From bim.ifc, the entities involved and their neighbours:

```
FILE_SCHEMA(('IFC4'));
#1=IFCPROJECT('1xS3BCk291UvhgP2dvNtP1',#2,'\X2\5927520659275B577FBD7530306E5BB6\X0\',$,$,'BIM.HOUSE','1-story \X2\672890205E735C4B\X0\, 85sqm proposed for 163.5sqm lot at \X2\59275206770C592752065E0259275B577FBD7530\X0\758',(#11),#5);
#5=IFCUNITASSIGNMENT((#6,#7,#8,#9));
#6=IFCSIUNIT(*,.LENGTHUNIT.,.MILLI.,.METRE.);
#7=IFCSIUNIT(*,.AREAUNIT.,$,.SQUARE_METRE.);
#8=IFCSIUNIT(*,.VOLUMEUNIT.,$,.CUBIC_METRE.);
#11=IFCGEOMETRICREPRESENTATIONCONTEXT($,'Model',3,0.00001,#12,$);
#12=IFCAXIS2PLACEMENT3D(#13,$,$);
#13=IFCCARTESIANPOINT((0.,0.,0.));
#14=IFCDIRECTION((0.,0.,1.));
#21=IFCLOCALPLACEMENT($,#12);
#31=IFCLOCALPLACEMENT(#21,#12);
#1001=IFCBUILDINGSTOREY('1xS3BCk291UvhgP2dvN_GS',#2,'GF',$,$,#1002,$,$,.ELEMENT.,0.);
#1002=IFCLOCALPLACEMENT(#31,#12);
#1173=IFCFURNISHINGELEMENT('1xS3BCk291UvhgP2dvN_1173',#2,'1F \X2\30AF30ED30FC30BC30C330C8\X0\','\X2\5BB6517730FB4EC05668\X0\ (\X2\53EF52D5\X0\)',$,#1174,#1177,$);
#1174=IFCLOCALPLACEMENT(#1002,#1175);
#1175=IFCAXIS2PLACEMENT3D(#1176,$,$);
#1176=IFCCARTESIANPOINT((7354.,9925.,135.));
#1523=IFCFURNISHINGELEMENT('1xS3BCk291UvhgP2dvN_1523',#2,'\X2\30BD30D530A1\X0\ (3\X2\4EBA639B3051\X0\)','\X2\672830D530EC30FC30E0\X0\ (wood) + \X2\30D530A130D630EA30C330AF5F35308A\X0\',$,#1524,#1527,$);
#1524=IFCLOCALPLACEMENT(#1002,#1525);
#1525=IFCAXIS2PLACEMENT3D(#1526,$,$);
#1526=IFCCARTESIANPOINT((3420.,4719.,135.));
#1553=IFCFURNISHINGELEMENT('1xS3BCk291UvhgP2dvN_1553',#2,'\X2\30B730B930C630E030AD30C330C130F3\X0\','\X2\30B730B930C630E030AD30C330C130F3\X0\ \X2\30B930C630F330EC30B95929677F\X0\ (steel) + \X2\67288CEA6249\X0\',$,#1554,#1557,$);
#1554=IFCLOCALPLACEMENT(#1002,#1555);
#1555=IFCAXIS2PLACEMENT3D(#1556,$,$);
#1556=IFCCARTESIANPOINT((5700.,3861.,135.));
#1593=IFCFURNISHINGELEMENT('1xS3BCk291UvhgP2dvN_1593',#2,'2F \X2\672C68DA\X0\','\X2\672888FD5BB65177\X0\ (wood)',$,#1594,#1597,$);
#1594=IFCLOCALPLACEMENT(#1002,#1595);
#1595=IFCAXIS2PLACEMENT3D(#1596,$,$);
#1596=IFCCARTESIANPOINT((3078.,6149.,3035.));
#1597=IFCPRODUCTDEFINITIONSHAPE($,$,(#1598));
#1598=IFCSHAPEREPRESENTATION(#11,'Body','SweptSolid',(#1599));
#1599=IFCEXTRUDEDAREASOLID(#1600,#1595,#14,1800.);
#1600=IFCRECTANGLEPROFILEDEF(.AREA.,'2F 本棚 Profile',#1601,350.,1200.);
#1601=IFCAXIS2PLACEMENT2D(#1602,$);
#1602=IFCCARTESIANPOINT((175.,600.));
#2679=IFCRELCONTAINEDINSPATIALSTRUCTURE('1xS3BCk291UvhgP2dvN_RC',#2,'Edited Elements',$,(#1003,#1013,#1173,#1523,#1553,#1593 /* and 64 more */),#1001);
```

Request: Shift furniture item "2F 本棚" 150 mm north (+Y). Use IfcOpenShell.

```python
import ifcopenshell
import ifcopenshell.api.geometry
import ifcopenshell.util.placement
import ifcopenshell.util.unit

model = ifcopenshell.open("bim.ifc")
unit_scale = ifcopenshell.util.unit.calculate_unit_scale(model)

item = model.by_guid("1xS3BCk291UvhgP2dvN_1593")
matrix = ifcopenshell.util.placement.get_local_placement(item.ObjectPlacement)
matrix[1, 3] += 0.15 / unit_scale
ifcopenshell.api.geometry.edit_object_placement(model, product=item, matrix=matrix, is_si=False)

print(ifcopenshell.util.placement.get_local_placement(item.ObjectPlacement).round(3) + 0.0)

model.write("bim_updated.ifc")
```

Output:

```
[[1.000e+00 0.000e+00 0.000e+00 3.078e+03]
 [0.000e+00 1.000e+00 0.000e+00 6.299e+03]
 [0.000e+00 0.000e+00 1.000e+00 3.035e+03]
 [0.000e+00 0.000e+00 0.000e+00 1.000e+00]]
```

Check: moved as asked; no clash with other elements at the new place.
